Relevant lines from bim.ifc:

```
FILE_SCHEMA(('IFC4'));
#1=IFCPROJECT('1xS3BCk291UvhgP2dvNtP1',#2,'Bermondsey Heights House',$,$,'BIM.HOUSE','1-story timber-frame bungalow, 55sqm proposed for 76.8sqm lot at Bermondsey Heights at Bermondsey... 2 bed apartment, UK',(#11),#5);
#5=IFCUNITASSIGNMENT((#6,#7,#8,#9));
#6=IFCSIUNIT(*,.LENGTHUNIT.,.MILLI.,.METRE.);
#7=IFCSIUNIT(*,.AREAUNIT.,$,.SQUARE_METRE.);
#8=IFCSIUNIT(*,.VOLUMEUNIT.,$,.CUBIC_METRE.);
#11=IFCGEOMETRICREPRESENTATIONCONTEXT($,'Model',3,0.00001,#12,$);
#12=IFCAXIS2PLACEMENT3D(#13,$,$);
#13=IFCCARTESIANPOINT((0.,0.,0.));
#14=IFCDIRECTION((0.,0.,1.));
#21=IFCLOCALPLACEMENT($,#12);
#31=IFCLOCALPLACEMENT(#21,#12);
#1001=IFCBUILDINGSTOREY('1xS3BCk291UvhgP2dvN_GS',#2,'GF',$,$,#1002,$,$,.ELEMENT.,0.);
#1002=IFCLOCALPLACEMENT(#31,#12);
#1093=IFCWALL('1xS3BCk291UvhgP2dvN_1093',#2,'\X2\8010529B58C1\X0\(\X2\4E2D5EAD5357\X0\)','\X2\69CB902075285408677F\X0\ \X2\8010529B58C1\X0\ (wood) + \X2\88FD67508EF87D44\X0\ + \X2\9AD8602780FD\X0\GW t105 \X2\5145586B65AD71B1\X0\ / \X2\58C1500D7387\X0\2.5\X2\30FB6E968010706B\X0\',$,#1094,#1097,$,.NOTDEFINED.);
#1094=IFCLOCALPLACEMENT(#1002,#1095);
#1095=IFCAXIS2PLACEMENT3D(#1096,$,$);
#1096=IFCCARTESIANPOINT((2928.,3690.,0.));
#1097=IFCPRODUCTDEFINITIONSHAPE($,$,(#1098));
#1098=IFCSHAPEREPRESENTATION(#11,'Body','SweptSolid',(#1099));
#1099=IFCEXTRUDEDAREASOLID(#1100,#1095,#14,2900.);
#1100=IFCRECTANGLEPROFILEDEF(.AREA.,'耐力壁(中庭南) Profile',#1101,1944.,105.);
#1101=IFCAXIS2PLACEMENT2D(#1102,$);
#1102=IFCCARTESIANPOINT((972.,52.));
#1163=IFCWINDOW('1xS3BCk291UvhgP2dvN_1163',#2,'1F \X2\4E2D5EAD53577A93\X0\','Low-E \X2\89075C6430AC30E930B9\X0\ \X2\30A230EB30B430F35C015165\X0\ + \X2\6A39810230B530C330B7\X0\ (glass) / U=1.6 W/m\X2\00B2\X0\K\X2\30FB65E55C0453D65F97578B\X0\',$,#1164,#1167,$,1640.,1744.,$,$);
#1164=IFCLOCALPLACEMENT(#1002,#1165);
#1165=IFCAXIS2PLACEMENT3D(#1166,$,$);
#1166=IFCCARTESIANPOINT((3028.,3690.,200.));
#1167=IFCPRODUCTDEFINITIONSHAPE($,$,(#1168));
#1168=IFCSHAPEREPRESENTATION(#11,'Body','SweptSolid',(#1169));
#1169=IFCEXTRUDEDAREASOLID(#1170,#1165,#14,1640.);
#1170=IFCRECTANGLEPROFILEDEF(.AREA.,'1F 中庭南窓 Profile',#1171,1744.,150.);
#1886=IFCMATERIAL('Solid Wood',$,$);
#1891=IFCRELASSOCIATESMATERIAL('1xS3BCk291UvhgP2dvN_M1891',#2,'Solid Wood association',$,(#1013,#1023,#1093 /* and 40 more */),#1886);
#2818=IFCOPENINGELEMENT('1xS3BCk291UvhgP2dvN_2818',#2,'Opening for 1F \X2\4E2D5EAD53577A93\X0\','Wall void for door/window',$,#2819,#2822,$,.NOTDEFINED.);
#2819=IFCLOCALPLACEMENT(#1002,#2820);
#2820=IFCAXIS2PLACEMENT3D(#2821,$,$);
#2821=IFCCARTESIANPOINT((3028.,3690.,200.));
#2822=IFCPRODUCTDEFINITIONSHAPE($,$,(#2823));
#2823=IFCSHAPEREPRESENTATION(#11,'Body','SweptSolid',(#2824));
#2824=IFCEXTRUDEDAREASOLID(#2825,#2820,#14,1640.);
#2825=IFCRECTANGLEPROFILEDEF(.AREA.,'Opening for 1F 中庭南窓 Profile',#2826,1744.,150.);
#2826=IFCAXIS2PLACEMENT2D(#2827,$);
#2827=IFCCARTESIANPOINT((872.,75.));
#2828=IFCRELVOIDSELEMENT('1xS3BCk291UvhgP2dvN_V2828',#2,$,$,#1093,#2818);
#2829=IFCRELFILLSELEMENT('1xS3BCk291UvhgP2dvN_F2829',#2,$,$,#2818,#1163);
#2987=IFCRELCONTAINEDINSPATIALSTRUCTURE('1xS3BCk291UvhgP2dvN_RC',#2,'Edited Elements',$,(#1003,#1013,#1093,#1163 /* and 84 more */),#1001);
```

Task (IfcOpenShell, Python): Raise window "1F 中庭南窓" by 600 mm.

```python
import numpy as np
import ifcopenshell
import ifcopenshell.api.geometry
import ifcopenshell.util.placement
import ifcopenshell.util.unit

model = ifcopenshell.open("bim.ifc")
unit_scale = ifcopenshell.util.unit.calculate_unit_scale(model)

window = model.by_guid("1xS3BCk291UvhgP2dvN_1163")
opening = window.FillsVoids[0].RelatingOpeningElement
dz = 0.6 / unit_scale

shift = np.array([0.0, 0.0, dz])
# The window is not placed relative to its opening, so move both.
for product in (opening, window):
    matrix = ifcopenshell.util.placement.get_local_placement(product.ObjectPlacement)
    matrix[:3, 3] += shift
    ifcopenshell.api.geometry.edit_object_placement(model, product=product, matrix=matrix, is_si=False)

print(f"moved by {dz * unit_scale:+.3f} m")

model.write("bim-out.ifc")
```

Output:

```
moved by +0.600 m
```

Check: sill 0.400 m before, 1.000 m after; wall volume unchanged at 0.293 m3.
